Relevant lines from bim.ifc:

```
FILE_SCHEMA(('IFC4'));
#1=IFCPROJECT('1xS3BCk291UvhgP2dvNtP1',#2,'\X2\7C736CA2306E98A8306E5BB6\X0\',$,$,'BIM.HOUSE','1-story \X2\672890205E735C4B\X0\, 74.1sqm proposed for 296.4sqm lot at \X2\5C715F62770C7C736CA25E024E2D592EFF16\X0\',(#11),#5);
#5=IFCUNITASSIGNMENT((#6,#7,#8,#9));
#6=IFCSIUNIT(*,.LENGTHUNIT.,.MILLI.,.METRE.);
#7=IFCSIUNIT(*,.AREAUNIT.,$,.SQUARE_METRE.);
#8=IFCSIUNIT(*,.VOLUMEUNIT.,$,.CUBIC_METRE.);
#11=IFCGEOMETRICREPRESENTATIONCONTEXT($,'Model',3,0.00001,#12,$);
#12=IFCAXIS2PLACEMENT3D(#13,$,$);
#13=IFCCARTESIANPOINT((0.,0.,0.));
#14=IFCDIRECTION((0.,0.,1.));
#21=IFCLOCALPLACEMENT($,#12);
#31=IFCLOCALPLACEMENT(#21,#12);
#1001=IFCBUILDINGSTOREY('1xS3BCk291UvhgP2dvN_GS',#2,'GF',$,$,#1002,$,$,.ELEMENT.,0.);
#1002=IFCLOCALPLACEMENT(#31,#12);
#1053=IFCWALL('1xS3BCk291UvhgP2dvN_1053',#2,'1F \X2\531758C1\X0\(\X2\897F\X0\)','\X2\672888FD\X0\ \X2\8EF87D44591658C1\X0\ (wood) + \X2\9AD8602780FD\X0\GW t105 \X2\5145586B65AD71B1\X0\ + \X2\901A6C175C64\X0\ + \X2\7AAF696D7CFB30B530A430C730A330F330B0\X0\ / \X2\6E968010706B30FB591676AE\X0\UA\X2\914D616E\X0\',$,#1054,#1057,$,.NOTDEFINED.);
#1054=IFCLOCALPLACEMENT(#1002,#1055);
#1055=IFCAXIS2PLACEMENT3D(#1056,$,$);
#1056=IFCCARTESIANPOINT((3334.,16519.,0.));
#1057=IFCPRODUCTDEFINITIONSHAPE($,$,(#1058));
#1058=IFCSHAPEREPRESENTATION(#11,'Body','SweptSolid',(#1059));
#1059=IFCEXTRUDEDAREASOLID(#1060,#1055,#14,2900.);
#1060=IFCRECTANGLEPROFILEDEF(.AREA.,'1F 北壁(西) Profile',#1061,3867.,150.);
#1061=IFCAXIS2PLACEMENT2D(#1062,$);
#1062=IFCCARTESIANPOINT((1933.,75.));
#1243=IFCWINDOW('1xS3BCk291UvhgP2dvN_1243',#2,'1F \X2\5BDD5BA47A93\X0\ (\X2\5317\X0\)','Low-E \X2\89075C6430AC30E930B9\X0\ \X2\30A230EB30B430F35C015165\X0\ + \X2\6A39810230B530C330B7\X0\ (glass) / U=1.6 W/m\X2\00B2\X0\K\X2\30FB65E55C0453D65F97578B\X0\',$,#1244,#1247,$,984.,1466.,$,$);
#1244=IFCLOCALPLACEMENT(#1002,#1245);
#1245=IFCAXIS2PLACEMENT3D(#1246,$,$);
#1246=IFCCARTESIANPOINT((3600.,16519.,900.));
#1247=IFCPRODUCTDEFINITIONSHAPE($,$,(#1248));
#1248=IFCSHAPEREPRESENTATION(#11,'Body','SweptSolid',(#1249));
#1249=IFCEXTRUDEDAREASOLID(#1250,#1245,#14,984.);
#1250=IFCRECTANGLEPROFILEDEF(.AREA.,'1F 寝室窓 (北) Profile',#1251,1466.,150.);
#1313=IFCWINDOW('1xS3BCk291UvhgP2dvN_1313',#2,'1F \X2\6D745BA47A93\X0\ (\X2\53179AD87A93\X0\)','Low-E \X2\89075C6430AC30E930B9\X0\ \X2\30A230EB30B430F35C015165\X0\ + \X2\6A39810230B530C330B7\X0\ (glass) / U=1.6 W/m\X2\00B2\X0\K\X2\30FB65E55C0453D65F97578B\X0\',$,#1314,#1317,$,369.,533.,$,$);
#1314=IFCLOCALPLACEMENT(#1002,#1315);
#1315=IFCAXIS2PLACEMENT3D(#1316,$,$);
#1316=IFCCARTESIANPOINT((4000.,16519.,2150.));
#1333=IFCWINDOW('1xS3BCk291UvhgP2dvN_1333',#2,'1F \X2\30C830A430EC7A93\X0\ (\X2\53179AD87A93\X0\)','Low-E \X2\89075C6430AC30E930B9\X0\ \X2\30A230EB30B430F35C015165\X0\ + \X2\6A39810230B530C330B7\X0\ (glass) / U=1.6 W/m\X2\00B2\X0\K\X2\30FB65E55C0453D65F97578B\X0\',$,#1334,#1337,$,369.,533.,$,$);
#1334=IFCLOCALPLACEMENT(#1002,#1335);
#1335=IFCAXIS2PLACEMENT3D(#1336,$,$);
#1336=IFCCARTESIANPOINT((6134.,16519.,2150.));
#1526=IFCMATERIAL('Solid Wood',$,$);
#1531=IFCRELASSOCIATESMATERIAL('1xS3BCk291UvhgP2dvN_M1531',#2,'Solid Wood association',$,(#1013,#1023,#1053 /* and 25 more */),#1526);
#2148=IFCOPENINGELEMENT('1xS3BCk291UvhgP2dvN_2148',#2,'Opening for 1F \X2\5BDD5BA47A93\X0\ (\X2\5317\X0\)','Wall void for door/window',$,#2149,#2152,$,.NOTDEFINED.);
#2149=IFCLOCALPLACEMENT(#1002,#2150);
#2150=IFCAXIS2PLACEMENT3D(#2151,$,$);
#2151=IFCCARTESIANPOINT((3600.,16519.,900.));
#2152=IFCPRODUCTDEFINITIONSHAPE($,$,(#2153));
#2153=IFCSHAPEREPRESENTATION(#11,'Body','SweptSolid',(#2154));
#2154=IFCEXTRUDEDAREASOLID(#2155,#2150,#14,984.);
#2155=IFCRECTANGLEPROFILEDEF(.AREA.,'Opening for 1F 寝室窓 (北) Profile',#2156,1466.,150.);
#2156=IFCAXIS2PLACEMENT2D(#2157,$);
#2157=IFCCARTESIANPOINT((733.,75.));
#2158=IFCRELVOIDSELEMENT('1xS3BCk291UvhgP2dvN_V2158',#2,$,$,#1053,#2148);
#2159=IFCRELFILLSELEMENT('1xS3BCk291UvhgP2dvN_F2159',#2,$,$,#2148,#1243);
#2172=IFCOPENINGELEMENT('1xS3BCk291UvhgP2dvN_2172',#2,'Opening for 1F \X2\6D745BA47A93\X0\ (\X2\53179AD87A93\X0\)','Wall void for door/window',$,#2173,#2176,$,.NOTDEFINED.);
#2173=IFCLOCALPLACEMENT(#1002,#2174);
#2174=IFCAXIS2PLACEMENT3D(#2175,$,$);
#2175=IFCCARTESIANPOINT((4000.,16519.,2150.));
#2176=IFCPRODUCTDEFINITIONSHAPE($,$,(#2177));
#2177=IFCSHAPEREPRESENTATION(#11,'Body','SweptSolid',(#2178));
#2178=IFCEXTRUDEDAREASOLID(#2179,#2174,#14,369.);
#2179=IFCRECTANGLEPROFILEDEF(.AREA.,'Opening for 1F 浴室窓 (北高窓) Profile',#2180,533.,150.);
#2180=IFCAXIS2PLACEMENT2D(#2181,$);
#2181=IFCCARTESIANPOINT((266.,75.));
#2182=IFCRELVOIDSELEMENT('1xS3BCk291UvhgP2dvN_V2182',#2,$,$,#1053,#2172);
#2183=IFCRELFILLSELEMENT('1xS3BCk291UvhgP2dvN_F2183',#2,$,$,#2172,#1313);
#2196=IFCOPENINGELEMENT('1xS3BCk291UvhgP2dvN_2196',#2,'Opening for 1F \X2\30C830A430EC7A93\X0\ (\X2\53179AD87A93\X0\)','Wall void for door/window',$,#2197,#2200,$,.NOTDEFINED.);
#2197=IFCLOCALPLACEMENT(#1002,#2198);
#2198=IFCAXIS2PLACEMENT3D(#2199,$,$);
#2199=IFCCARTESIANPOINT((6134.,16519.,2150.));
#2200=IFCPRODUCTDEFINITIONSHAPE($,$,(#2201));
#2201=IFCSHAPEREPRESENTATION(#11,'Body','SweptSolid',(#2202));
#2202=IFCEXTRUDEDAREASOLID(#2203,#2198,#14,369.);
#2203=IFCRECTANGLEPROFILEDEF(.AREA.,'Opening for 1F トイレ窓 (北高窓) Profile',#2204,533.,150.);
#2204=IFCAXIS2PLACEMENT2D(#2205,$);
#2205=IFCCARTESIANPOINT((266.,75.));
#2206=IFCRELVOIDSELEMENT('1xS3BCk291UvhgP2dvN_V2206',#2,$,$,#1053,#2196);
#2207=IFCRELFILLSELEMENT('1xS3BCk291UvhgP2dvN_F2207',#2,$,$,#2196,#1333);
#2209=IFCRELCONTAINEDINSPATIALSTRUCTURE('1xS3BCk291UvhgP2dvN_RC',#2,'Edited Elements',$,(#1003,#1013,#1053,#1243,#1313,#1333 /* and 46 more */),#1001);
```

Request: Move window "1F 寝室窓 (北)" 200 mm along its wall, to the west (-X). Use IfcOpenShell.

```python
import ifcopenshell
import ifcopenshell.api.geometry
import ifcopenshell.util.placement

model = ifcopenshell.open("bim.ifc")

window = model.by_id(1243)
opening = window.FillsVoids[0].RelatingOpeningElement
wall = opening.VoidsElements[0].RelatingBuildingElement

wall_matrix = ifcopenshell.util.placement.get_local_placement(wall.ObjectPlacement)
shift = wall_matrix[:3, 0] * -200.0
before = ifcopenshell.util.placement.get_local_placement(window.ObjectPlacement)[:3, 3].copy()

# The window is not placed relative to its opening, so move both.
for product in (opening, window):
    matrix = ifcopenshell.util.placement.get_local_placement(product.ObjectPlacement)
    matrix[:3, 3] += shift
    ifcopenshell.api.geometry.edit_object_placement(model, product=product, matrix=matrix, is_si=False)

after = ifcopenshell.util.placement.get_local_placement(window.ObjectPlacement)[:3, 3]
print("window moved by", (after - before).round(3) + 0.0)

model.write("bim_v2.ifc")
```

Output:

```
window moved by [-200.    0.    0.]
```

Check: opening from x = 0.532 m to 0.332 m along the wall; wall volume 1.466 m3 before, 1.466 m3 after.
